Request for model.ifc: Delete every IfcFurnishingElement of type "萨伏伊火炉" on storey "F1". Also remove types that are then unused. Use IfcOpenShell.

First a look at what the model holds.

```python
import ifcopenshell
import ifcopenshell.util.element

model = ifcopenshell.open("model.ifc")
print(model.schema)
storey = next(s for s in model.by_type("IfcBuildingStorey") if s.Name == "F1")
furniture = [e for e in ifcopenshell.util.element.get_decomposition(storey) if e.is_a("IfcFurnishingElement")]
seen = {}
for e in furniture:
    element_type = ifcopenshell.util.element.get_type(e)
    name = element_type.Name if element_type not in (None, e) else None
    seen[name] = seen.get(name, 0) + 1
for name, count in sorted(seen.items(), key=str):
    print(count, "x", name)
```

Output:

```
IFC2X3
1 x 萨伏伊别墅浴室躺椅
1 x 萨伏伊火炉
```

```python
import ifcopenshell
import ifcopenshell.api.root
import ifcopenshell.util.element

model = ifcopenshell.open("model.ifc")

storey = next(s for s in model.by_type("IfcBuildingStorey") if s.Name == "F1")
furniture = [e for e in ifcopenshell.util.element.get_decomposition(storey) if e.is_a("IfcFurnishingElement")]
targets = [e for e in furniture if (t := ifcopenshell.util.element.get_type(e)) not in (None, e) and t.Name == "萨伏伊火炉"]
types = {ifcopenshell.util.element.get_type(e) for e in targets} - {None, *targets}

for e in targets:
    ifcopenshell.api.root.remove_product(model, product=e)
print(len(targets), "removed")

unused = [t for t in types if not ifcopenshell.util.element.get_types(t)]
for t in unused:
    ifcopenshell.api.root.remove_product(model, product=t)
print(len(unused), "unused types removed")

model.write("model_rev.ifc")
```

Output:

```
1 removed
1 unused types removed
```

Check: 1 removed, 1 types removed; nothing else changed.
